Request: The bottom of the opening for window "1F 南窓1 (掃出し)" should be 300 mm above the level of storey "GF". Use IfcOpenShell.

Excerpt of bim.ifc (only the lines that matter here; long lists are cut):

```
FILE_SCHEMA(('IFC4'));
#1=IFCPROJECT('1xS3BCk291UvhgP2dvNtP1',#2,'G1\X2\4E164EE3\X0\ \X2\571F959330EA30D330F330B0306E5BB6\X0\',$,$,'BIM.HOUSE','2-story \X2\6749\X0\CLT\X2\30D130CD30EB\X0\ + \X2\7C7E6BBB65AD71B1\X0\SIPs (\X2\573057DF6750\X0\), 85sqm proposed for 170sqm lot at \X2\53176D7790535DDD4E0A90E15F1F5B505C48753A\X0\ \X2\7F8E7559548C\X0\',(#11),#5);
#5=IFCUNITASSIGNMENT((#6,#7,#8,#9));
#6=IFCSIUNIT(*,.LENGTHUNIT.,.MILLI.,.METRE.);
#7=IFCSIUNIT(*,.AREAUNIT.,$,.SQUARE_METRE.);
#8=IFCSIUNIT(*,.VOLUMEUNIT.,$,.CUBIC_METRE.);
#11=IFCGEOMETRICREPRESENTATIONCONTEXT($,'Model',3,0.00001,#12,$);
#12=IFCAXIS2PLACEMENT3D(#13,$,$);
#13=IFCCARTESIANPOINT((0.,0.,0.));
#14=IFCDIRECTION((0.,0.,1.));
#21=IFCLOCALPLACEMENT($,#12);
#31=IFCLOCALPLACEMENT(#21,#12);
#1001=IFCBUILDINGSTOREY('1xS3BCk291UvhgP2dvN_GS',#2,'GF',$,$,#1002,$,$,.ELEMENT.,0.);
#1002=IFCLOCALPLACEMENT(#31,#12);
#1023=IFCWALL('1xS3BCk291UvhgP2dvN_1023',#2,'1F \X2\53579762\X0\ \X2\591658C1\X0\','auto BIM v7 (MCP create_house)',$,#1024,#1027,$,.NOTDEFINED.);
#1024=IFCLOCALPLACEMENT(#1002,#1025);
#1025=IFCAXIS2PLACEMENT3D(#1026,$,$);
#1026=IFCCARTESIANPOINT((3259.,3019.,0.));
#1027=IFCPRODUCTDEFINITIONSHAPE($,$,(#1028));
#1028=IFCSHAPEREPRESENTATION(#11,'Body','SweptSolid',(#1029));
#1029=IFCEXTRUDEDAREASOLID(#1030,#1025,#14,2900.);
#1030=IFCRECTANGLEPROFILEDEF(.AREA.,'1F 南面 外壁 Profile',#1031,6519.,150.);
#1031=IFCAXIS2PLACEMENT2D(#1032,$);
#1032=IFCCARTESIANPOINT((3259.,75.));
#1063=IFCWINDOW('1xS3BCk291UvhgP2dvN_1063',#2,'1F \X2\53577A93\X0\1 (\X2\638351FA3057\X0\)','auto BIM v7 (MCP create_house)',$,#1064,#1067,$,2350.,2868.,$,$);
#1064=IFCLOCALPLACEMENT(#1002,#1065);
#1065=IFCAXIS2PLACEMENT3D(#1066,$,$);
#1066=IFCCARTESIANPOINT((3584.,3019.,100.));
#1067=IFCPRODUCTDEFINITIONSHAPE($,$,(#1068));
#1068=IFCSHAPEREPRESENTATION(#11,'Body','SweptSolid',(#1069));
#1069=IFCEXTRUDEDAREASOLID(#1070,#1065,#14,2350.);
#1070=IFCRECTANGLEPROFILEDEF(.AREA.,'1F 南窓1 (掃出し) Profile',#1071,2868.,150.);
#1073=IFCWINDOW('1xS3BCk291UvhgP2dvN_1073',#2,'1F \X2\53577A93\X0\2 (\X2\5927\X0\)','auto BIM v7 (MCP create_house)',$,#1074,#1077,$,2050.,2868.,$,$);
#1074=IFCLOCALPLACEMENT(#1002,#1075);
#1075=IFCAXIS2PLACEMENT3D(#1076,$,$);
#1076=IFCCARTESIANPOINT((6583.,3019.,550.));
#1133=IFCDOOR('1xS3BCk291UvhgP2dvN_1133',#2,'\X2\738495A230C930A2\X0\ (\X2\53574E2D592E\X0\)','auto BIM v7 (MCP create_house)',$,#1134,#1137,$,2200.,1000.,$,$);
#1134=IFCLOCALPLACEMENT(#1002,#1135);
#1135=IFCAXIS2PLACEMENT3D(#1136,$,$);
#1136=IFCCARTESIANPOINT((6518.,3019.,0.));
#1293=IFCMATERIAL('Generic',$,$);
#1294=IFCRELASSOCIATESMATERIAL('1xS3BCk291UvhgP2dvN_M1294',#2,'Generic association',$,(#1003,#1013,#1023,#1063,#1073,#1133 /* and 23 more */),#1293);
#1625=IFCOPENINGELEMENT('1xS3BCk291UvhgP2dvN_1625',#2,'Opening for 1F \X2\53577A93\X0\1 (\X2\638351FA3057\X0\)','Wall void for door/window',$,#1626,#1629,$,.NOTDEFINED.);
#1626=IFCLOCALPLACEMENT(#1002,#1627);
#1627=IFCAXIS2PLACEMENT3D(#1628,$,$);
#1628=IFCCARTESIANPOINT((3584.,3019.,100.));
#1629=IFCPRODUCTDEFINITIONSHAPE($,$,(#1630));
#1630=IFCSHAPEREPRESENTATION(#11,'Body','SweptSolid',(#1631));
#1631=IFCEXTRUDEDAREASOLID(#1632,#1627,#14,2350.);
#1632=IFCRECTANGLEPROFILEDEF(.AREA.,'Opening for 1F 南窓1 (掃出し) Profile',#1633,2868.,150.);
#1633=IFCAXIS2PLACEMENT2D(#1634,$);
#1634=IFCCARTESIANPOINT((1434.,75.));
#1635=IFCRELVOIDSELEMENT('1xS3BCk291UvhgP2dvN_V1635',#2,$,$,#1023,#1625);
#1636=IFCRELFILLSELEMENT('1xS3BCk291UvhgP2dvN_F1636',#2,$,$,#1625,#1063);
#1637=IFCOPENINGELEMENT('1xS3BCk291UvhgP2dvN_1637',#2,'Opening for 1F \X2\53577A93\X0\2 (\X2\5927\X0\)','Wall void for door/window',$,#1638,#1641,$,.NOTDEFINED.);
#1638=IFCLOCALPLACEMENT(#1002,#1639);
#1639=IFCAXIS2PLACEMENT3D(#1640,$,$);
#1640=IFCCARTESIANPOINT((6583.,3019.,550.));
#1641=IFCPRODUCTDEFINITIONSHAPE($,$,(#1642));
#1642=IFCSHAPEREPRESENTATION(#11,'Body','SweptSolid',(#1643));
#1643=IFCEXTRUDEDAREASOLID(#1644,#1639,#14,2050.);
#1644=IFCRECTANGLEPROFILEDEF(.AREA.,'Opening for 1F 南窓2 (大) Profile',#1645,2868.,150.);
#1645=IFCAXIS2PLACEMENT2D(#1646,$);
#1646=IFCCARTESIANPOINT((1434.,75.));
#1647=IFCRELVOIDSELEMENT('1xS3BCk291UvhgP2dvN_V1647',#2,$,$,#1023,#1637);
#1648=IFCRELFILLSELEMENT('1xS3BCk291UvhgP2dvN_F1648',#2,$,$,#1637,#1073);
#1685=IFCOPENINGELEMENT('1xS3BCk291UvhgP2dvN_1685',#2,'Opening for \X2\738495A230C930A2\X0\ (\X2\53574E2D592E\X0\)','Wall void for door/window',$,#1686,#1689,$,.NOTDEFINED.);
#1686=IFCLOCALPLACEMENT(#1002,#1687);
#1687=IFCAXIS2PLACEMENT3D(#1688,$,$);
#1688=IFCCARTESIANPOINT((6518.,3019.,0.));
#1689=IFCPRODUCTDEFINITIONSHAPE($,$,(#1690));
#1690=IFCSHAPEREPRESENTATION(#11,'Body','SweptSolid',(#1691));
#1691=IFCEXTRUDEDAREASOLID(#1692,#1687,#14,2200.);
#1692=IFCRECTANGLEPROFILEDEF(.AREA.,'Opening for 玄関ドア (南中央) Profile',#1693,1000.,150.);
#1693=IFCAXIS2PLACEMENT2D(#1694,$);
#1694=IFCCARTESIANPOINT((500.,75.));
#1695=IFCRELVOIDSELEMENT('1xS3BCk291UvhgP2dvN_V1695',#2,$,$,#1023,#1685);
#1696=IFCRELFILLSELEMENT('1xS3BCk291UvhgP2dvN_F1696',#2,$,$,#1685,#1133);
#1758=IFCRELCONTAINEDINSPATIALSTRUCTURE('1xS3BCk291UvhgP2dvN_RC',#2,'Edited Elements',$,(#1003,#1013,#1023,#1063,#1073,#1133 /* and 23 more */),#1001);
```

```python
import numpy as np
import ifcopenshell
import ifcopenshell.api.geometry
import ifcopenshell.geom
import ifcopenshell.util.element
import ifcopenshell.util.placement
import ifcopenshell.util.shape
import ifcopenshell.util.unit

model = ifcopenshell.open("bim.ifc")
unit_scale = ifcopenshell.util.unit.calculate_unit_scale(model)

window = model.by_id(1063)
opening = window.FillsVoids[0].RelatingOpeningElement
storey = ifcopenshell.util.element.get_container(window, ifc_class="IfcBuildingStorey")
level = ifcopenshell.util.placement.get_local_placement(storey.ObjectPlacement)[2, 3]

# The opening's origin need not be at the sill, so measure its lowest point.
shape = ifcopenshell.geom.create_shape(ifcopenshell.geom.settings(), opening)
bottom = ifcopenshell.util.shape.get_shape_bottom_elevation(shape, shape.geometry) / unit_scale
dz = level + 300.0 - bottom

shift = np.array([0.0, 0.0, dz])
# The window is not placed relative to its opening, so move both.
for product in (opening, window):
    matrix = ifcopenshell.util.placement.get_local_placement(product.ObjectPlacement)
    matrix[:3, 3] += shift
    ifcopenshell.api.geometry.edit_object_placement(model, product=product, matrix=matrix, is_si=False)

print(f"moved by {dz * unit_scale:+.3f} m")

model.write("bim_edited.ifc")
```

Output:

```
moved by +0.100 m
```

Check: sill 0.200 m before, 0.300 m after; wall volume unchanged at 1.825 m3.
